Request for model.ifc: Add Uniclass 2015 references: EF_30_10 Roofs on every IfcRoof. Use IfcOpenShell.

First a look at what the model holds.

```python
import ifcopenshell

model = ifcopenshell.open("model.ifc")
print(model.schema)
print("classifications:", [c.Name for c in model.by_type("IfcClassification")])
for ifc_class in ("IfcDoor", "IfcRoof", "IfcStair", "IfcWall", "IfcWindow"):
    print(ifc_class, len(model.by_type(ifc_class)))
```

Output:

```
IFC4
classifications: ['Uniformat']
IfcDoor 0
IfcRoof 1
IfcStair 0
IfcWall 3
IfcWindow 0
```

```python
import ifcopenshell
import ifcopenshell.api.classification

model = ifcopenshell.open("model.ifc")

system = ifcopenshell.api.classification.add_classification(model, classification="Uniclass 2015")

codes = {
    "IfcRoof": ("EF_30_10", "Roofs"),
}
for ifc_class, (code, name) in codes.items():
    products = model.by_type(ifc_class)
    ifcopenshell.api.classification.add_reference(
        model, products=products, classification=system, identification=code, name=name
    )
    print(code, len(products))

model.write("model_edited.ifc")
```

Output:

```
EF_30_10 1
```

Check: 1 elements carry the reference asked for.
